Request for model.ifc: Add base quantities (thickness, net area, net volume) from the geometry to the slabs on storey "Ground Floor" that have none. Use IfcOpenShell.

First a look at what the model holds.

```python
import ifcopenshell
import ifcopenshell.util.element
import ifcopenshell.util.unit

model = ifcopenshell.open("model.ifc")
print(model.schema)
for unit_type in ("LENGTHUNIT", "AREAUNIT", "VOLUMEUNIT"):
    print(unit_type, ifcopenshell.util.unit.calculate_unit_scale(model, unit_type))
storey = next(s for s in model.by_type("IfcBuildingStorey") if s.Name == "Ground Floor")
slabs = [e for e in ifcopenshell.util.element.get_decomposition(storey) if e.is_a("IfcSlab")]
for e in sorted(slabs, key=lambda e: e.id()):
    print(e.id(), e.is_a(), e.Name, list(ifcopenshell.util.element.get_psets(e, qtos_only=True)), sep=" | ")
```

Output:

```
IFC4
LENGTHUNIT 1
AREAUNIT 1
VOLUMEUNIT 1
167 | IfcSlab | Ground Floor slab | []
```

```python
import ifcopenshell
import ifcopenshell.api.pset
import ifcopenshell.geom
import ifcopenshell.util.element
import ifcopenshell.util.shape
import ifcopenshell.util.unit

model = ifcopenshell.open("model.ifc")
unit_scale = ifcopenshell.util.unit.calculate_unit_scale(model)
area_scale = ifcopenshell.util.unit.calculate_unit_scale(model, "AREAUNIT")
volume_scale = ifcopenshell.util.unit.calculate_unit_scale(model, "VOLUMEUNIT")
settings = ifcopenshell.geom.settings()

storey = next(s for s in model.by_type("IfcBuildingStorey") if s.Name == "Ground Floor")
slabs = [e for e in ifcopenshell.util.element.get_decomposition(storey) if e.is_a("IfcSlab")]

for e in sorted(slabs, key=lambda e: e.id()):
    if ifcopenshell.util.element.get_psets(e, qtos_only=True, should_inherit=False):
        continue
    # Geometry comes back in metres, in the element's own axes.
    shape = ifcopenshell.geom.create_shape(settings, e)
    values = {
        "Width": ifcopenshell.util.shape.get_z(shape.geometry) / unit_scale,
        "NetArea": ifcopenshell.util.shape.get_footprint_area(shape.geometry) / area_scale,
        "NetVolume": ifcopenshell.util.shape.get_volume(shape.geometry) / volume_scale,
    }
    qto = ifcopenshell.api.pset.add_qto(model, product=e, name="Qto_SlabBaseQuantities")
    ifcopenshell.api.pset.edit_qto(model, qto=qto, properties=values)
    print(e.id(), {k: round(v, 3) for k, v in values.items()})

model.write("model_edited.ifc")
```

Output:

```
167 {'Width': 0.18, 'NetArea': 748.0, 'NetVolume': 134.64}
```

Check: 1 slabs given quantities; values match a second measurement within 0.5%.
